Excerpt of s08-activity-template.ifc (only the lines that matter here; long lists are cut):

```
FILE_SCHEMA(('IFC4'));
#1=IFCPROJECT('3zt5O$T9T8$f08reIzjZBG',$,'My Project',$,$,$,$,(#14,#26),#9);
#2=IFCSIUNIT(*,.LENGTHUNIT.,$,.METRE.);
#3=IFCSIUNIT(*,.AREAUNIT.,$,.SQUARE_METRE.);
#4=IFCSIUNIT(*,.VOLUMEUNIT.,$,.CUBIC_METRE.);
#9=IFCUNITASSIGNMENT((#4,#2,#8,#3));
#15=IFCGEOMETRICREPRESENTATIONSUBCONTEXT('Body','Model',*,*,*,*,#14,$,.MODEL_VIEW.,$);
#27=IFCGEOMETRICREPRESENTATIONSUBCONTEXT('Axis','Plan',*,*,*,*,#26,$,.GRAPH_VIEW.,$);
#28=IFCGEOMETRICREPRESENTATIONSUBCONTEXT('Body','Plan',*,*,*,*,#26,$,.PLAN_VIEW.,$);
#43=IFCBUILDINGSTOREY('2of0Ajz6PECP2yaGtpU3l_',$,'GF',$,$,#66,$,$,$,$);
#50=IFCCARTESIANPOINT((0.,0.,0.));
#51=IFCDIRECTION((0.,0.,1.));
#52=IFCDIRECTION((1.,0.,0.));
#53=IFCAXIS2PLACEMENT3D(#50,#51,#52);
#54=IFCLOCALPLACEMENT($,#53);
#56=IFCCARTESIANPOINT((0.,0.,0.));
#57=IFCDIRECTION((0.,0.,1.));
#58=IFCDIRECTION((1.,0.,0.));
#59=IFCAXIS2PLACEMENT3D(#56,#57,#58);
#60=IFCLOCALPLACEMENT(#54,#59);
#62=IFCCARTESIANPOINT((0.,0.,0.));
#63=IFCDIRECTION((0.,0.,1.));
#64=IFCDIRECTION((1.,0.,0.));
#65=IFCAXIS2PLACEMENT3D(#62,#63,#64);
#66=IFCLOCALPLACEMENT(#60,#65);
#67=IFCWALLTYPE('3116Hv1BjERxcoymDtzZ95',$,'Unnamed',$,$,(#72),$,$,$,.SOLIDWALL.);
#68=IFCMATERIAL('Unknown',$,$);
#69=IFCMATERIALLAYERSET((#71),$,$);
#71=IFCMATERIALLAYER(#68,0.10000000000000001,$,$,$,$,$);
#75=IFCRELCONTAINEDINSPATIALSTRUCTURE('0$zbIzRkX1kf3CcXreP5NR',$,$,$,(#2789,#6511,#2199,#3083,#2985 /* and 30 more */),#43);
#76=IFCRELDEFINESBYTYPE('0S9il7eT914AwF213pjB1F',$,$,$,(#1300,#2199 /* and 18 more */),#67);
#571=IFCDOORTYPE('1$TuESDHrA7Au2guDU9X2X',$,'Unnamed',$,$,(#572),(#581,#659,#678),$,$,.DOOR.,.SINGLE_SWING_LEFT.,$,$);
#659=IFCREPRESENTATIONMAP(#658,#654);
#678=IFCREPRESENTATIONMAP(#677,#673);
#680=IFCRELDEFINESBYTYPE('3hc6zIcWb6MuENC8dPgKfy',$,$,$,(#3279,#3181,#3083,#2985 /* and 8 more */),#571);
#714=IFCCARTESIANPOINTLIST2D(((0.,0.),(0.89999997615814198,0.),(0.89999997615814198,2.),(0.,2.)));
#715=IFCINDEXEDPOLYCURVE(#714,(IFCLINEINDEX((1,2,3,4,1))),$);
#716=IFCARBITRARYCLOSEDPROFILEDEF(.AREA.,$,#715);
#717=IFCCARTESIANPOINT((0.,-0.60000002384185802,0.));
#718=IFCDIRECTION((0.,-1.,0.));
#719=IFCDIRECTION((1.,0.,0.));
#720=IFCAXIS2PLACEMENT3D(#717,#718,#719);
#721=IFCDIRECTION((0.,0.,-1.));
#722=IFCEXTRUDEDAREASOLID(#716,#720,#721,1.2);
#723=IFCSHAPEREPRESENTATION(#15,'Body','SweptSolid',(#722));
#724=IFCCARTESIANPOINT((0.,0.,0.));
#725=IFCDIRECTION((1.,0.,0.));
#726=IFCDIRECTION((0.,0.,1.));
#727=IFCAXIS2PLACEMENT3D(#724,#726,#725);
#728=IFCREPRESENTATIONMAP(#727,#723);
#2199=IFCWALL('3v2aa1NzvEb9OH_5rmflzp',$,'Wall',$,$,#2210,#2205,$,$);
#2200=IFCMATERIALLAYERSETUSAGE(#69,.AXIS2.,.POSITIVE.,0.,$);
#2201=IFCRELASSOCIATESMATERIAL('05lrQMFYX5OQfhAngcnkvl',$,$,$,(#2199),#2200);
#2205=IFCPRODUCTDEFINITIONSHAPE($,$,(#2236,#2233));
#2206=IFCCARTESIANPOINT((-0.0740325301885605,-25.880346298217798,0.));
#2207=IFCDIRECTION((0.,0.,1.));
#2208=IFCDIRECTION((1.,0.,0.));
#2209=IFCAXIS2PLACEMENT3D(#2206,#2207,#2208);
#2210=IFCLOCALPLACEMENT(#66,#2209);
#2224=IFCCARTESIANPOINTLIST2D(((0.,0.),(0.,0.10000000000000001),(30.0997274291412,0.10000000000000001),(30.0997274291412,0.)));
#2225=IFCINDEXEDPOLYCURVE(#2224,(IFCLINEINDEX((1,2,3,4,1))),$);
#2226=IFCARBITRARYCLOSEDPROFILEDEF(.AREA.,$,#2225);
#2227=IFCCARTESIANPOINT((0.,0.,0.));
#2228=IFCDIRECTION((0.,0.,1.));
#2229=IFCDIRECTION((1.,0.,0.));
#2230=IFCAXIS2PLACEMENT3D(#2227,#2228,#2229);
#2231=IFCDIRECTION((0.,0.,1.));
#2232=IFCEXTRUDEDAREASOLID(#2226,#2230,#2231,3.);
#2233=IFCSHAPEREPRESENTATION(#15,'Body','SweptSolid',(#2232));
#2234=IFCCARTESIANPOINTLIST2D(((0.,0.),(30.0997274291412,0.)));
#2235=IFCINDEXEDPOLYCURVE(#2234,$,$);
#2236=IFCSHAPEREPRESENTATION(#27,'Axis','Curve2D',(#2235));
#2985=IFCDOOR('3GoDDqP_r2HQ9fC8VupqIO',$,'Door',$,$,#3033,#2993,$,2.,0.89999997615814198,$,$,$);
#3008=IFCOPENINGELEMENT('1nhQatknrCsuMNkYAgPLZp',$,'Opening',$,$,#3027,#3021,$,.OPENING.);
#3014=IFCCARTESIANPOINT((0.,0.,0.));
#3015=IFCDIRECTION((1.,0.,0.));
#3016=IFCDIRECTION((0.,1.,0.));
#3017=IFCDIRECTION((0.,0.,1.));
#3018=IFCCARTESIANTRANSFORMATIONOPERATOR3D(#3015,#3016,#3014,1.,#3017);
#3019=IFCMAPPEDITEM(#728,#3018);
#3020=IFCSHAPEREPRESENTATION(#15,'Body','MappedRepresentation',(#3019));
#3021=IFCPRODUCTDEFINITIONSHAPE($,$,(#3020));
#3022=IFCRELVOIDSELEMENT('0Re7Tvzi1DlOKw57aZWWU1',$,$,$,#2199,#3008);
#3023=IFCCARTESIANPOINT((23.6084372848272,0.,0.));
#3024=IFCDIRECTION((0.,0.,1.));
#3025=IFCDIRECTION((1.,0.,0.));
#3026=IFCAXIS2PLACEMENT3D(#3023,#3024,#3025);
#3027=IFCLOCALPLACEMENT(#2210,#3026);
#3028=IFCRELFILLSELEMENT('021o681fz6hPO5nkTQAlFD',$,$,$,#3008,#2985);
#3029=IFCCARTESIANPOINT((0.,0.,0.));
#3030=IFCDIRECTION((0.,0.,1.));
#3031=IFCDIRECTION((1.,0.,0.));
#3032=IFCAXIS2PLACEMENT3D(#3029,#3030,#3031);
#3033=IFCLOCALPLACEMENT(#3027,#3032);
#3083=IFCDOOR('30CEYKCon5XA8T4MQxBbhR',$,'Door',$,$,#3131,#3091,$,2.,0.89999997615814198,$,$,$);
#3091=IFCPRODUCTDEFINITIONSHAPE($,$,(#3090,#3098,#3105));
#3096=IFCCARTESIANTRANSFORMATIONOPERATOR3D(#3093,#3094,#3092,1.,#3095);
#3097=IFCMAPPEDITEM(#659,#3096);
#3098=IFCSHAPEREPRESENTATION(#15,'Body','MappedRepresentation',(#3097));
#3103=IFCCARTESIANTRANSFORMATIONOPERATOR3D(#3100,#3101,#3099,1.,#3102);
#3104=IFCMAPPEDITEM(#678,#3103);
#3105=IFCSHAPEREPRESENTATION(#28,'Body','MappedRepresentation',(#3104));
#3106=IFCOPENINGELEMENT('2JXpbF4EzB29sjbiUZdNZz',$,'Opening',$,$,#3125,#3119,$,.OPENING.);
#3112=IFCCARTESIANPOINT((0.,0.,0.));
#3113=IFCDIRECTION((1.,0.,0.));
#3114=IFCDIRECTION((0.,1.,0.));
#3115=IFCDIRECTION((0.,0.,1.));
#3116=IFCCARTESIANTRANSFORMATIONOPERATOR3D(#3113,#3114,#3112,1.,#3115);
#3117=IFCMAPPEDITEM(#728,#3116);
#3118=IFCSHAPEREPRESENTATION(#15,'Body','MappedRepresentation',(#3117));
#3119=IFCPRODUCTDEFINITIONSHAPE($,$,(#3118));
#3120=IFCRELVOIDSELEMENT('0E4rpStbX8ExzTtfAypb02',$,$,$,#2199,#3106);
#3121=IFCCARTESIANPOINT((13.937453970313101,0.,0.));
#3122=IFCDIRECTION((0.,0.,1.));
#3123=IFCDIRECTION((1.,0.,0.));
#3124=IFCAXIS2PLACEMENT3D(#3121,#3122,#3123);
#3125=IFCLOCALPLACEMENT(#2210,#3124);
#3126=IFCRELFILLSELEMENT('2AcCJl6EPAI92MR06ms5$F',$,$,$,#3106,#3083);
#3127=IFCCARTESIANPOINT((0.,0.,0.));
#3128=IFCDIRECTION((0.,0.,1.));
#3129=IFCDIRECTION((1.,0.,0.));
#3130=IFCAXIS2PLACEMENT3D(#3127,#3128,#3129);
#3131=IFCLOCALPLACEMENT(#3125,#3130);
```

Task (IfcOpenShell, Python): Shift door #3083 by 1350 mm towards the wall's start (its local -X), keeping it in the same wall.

```python
import ifcopenshell
import ifcopenshell.api.geometry
import ifcopenshell.util.placement

model = ifcopenshell.open("s08-activity-template.ifc")

door = model.by_guid("30CEYKCon5XA8T4MQxBbhR")
opening = door.FillsVoids[0].RelatingOpeningElement
wall = opening.VoidsElements[0].RelatingBuildingElement

wall_matrix = ifcopenshell.util.placement.get_local_placement(wall.ObjectPlacement)
shift = wall_matrix[:3, 0] * -1.35
before = ifcopenshell.util.placement.get_local_placement(door.ObjectPlacement)[:3, 3].copy()

# The door is placed relative to its opening, so it follows when the opening moves.
matrix = ifcopenshell.util.placement.get_local_placement(opening.ObjectPlacement)
matrix[:3, 3] += shift
ifcopenshell.api.geometry.edit_object_placement(
    model, product=opening, matrix=matrix, is_si=False, should_transform_children=True
)

after = ifcopenshell.util.placement.get_local_placement(door.ObjectPlacement)[:3, 3]
print("door moved by", (after - before).round(3) + 0.0)

model.write("s08-activity-template_rev.ifc")
```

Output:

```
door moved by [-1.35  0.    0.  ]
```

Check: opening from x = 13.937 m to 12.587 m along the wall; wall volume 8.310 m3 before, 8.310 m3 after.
